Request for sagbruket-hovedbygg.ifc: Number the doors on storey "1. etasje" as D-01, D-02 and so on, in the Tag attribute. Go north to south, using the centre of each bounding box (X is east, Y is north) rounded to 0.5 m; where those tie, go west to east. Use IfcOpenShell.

First a look at what the model holds.

```python
import ifcopenshell
import ifcopenshell.util.element
import ifcopenshell.util.placement

model = ifcopenshell.open("sagbruket-hovedbygg.ifc")
print(model.schema)
storey = next(s for s in model.by_type("IfcBuildingStorey") if s.Name == "1. etasje")
doors = [e for e in ifcopenshell.util.element.get_decomposition(storey) if e.is_a("IfcDoor")]
for e in sorted(doors, key=lambda e: e.id()):
    origin = ifcopenshell.util.placement.get_local_placement(e.ObjectPlacement)[:3, 3]
    print(e.id(), e.Tag, e.Name, origin.round(2) + 0.0, sep=" | ")
```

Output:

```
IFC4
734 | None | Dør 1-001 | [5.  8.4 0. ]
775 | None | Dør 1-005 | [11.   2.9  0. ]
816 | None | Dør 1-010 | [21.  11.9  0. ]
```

```python
import ifcopenshell
import ifcopenshell.geom
import ifcopenshell.util.element
import ifcopenshell.util.shape

model = ifcopenshell.open("sagbruket-hovedbygg.ifc")
settings = ifcopenshell.geom.settings()
settings.set("use-world-coords", True)


def centre(element):
    shape = ifcopenshell.geom.create_shape(settings, element)
    return ifcopenshell.util.shape.get_bbox_centroid(shape.geometry)


storey = next(s for s in model.by_type("IfcBuildingStorey") if s.Name == "1. etasje")
doors = [e for e in ifcopenshell.util.element.get_decomposition(storey) if e.is_a("IfcDoor")]

# Insertion points can sit at a corner or the storey origin, so sort by the geometry (in metres).
centres = {e: centre(e) for e in doors}
doors.sort(key=lambda e: (-round(centres[e][1] / 0.5), centres[e][0]))

for i, e in enumerate(doors, start=1):
    number = f"D-{i:02d}"
    e.Tag = number
    print(e.id(), number)

model.write("sagbruket-hovedbygg-out.ifc")
```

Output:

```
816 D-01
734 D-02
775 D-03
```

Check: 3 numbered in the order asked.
